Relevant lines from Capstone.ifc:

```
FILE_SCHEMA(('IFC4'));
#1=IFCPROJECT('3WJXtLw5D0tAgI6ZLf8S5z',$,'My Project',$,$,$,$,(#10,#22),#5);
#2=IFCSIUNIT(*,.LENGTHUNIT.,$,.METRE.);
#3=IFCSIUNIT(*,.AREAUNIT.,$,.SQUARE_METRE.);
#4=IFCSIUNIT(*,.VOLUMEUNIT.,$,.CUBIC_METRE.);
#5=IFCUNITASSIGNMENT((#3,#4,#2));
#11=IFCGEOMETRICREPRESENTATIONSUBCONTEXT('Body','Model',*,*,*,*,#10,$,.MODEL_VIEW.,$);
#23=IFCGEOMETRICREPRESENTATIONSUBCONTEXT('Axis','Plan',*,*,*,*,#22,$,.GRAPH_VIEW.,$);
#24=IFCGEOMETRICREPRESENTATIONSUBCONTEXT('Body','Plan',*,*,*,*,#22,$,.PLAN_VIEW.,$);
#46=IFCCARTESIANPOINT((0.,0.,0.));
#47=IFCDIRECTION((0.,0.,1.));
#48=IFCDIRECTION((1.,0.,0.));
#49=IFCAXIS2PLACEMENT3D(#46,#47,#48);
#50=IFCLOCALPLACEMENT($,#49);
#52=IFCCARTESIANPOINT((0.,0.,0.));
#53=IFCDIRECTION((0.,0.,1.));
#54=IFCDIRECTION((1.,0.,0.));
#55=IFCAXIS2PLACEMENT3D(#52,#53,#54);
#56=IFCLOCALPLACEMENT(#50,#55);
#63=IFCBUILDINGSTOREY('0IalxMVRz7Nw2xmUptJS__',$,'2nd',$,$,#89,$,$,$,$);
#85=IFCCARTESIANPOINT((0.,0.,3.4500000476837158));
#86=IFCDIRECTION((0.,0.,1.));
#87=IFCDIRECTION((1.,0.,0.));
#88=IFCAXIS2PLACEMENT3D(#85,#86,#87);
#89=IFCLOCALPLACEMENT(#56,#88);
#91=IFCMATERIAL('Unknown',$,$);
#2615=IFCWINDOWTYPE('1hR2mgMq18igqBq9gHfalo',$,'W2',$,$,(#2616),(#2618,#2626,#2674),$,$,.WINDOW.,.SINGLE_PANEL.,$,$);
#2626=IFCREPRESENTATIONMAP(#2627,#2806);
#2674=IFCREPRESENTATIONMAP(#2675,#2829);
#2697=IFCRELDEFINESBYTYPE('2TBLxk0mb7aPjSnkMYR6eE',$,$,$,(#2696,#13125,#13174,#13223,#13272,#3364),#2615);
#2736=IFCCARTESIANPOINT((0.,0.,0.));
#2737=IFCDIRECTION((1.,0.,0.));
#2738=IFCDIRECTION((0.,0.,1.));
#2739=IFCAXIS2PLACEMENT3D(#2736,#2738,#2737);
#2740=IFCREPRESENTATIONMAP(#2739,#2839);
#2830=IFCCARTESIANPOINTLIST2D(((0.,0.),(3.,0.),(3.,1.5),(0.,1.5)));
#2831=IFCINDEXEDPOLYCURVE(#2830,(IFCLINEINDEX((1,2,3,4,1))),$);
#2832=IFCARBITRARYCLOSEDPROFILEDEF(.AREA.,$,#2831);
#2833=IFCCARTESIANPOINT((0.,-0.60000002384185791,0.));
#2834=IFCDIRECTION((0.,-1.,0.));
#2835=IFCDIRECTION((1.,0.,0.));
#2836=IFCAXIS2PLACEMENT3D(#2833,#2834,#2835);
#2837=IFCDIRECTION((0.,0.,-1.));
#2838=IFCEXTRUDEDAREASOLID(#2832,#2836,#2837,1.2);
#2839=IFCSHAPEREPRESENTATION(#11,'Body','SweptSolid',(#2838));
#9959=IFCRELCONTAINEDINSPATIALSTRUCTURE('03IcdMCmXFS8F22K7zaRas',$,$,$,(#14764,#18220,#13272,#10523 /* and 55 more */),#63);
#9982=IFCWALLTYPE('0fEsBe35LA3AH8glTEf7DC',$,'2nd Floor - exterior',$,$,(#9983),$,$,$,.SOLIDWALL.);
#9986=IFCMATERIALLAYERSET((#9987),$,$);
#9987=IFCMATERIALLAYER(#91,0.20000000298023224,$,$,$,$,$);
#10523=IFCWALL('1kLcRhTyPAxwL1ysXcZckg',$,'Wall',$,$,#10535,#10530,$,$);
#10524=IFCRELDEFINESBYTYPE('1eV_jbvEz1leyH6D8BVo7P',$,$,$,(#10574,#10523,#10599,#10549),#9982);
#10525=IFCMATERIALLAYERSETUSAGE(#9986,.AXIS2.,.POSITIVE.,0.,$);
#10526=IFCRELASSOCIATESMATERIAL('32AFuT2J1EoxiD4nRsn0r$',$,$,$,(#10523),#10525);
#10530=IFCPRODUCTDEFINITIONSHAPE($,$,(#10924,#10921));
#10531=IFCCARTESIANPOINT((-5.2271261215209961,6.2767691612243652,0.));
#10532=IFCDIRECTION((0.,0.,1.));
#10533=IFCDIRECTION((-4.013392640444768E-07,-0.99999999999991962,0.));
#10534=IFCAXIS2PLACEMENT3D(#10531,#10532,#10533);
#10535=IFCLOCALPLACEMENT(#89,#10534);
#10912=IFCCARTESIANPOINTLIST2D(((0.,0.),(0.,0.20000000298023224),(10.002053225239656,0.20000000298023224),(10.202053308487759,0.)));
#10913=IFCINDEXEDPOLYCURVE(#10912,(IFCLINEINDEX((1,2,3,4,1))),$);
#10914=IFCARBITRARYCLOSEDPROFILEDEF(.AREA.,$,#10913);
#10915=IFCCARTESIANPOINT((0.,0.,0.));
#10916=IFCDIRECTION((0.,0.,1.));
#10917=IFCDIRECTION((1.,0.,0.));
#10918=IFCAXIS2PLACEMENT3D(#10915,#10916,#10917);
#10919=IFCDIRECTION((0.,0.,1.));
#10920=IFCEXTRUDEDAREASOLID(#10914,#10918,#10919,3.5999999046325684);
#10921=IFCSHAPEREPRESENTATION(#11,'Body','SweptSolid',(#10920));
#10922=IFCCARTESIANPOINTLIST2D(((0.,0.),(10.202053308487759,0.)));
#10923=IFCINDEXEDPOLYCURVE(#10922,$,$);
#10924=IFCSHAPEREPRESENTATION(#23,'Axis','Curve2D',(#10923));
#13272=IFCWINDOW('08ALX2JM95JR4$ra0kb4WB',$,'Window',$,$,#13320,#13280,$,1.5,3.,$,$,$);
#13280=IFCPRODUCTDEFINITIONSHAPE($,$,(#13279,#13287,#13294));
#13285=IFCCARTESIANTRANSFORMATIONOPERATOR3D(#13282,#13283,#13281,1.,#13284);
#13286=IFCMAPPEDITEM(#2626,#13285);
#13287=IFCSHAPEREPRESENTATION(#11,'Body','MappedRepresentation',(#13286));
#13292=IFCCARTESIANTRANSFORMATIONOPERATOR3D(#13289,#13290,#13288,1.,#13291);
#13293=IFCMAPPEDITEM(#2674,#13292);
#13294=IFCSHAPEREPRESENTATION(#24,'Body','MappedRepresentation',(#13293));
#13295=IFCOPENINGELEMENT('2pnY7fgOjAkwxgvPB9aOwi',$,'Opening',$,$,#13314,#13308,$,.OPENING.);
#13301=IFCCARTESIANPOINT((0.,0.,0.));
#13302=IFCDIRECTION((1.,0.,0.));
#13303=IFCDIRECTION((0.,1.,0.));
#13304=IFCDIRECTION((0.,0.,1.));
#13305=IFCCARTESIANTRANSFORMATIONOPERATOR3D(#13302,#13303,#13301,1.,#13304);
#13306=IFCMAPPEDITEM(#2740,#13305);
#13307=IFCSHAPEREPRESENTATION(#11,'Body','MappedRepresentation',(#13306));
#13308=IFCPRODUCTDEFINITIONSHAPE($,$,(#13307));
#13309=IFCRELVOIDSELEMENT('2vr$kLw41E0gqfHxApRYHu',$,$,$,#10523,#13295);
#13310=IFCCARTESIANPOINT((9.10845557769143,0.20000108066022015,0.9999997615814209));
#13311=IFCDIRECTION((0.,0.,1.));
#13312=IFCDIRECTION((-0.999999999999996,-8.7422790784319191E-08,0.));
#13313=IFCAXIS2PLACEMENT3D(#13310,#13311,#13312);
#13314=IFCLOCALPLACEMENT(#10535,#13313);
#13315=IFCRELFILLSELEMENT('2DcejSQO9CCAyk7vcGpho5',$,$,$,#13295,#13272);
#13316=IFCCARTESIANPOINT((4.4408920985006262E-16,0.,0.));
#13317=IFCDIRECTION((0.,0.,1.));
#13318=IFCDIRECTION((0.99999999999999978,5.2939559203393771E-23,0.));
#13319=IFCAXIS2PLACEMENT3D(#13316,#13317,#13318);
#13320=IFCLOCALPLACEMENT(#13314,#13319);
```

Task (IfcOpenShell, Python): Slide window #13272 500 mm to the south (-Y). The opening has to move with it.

```python
import ifcopenshell
import ifcopenshell.api.geometry
import ifcopenshell.util.placement

model = ifcopenshell.open("Capstone.ifc")

window = model.by_guid("08ALX2JM95JR4$ra0kb4WB")
opening = window.FillsVoids[0].RelatingOpeningElement
wall = opening.VoidsElements[0].RelatingBuildingElement

wall_matrix = ifcopenshell.util.placement.get_local_placement(wall.ObjectPlacement)
shift = wall_matrix[:3, 0] * 0.5
before = ifcopenshell.util.placement.get_local_placement(window.ObjectPlacement)[:3, 3].copy()

# The window is placed relative to its opening, so it follows when the opening moves.
matrix = ifcopenshell.util.placement.get_local_placement(opening.ObjectPlacement)
matrix[:3, 3] += shift
ifcopenshell.api.geometry.edit_object_placement(
    model, product=opening, matrix=matrix, is_si=False, should_transform_children=True
)

after = ifcopenshell.util.placement.get_local_placement(window.ObjectPlacement)[:3, 3]
print("window moved by", (after - before).round(3) + 0.0)

model.write("Capstone_updated.ifc")
```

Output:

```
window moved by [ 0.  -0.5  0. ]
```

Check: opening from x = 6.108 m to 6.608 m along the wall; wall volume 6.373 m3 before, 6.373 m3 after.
